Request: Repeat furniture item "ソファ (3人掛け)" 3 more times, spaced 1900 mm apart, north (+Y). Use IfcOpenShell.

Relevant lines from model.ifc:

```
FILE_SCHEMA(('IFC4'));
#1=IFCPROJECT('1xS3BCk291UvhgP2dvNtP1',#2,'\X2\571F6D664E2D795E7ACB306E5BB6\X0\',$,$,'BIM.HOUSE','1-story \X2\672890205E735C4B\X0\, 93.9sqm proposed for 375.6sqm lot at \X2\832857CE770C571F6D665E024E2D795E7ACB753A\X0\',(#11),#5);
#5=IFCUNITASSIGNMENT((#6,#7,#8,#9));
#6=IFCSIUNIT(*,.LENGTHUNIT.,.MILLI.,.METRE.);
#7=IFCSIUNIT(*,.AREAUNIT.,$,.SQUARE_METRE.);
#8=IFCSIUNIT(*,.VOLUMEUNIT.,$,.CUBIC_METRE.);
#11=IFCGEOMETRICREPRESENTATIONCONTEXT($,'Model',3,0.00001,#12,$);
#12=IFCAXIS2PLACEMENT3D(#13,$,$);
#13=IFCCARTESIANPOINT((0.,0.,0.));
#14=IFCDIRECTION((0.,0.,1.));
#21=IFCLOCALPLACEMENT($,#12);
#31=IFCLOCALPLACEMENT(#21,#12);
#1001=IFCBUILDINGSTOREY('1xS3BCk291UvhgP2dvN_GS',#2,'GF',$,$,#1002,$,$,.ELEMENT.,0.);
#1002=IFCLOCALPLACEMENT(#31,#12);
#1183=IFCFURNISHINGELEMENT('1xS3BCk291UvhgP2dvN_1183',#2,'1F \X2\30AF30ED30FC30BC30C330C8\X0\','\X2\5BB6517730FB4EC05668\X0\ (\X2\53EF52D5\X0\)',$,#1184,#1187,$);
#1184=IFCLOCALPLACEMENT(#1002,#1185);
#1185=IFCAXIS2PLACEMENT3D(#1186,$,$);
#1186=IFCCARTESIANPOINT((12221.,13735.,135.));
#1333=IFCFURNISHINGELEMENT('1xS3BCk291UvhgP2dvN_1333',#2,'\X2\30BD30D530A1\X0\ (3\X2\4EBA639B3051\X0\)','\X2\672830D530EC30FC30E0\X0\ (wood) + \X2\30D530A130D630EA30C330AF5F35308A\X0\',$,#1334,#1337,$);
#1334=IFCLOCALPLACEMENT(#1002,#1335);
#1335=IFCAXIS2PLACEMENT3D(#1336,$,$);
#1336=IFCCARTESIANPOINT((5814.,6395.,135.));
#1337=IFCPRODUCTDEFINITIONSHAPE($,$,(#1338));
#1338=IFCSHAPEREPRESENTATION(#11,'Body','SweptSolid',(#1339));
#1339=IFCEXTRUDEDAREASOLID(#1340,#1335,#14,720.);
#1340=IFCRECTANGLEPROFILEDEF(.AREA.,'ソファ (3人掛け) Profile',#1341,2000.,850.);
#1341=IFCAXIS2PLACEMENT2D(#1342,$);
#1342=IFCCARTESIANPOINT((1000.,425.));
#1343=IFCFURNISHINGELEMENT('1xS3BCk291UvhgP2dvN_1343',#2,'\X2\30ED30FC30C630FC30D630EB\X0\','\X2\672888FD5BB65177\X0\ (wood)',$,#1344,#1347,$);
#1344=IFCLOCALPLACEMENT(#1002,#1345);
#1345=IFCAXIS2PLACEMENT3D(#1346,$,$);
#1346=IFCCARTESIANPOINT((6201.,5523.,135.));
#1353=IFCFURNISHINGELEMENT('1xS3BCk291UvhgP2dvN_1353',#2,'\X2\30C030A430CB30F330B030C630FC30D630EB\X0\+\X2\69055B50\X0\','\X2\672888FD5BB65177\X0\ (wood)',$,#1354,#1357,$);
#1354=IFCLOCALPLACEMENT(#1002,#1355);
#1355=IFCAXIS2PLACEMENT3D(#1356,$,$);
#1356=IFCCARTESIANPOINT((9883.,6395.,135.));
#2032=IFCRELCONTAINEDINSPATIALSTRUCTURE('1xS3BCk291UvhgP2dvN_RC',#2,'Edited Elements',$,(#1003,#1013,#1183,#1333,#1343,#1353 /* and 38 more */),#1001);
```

```python
import numpy as np
import ifcopenshell
import ifcopenshell.api.geometry
import ifcopenshell.api.root
import ifcopenshell.util.element
import ifcopenshell.util.placement

model = ifcopenshell.open("model.ifc")


def reuse_history(source, copy):
    """copy_class also copies each property set's owner history, people and application; keep the originals."""
    for rel in copy.IsDefinedBy:
        if rel.is_a("IfcRelDefinesByProperties") and (history := rel.RelatingPropertyDefinition.OwnerHistory):
            rel.RelatingPropertyDefinition.OwnerHistory = source.OwnerHistory
            ifcopenshell.util.element.remove_deep2(model, history)


source = model.by_guid("1xS3BCk291UvhgP2dvN_1333")
base = ifcopenshell.util.placement.get_local_placement(source.ObjectPlacement)
step = np.array([0.0, 1.0, 0.0]) * 1900.0

for i in range(1, 4):
    copy = ifcopenshell.api.root.copy_class(model, product=source)
    copy.Representation = ifcopenshell.util.element.copy_deep(
        model, source.Representation, exclude=["IfcGeometricRepresentationContext", "IfcRepresentationMap"]
    )
    reuse_history(source, copy)
    matrix = base.copy()
    matrix[:3, 3] += i * step
    print("added at", matrix[:3, 3].round(3) + 0.0)
    ifcopenshell.api.geometry.edit_object_placement(model, product=copy, matrix=matrix, is_si=False)

model.write("model_edited.ifc")
```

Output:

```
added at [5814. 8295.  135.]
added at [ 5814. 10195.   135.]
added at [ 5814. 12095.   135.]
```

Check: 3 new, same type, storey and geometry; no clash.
